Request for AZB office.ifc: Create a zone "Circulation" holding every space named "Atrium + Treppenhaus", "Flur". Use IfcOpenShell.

First a look at what the model holds.

```python
import ifcopenshell

model = ifcopenshell.open("AZB office.ifc")
print(model.schema)
seen = {}
for space in model.by_type("IfcSpace"):
    seen[space.LongName] = seen.get(space.LongName, 0) + 1
for name, count in sorted(seen.items(), key=str):
    print(count, "x", name)
print("zones:", [z.Name for z in model.by_type("IfcZone")][:20])
```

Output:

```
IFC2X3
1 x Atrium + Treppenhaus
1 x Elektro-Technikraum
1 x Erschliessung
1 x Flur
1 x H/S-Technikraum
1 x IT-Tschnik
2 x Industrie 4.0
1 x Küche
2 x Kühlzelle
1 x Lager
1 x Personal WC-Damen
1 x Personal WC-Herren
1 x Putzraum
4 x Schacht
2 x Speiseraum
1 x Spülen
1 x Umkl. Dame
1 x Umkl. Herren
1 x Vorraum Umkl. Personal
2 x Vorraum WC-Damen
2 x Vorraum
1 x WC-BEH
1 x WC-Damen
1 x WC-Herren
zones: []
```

```python
import ifcopenshell
import ifcopenshell.api.group
import ifcopenshell.api.root

model = ifcopenshell.open("AZB office.ifc")

names = {"Atrium + Treppenhaus", "Flur"}
spaces = [s for s in model.by_type("IfcSpace") if s.LongName in names]

zone = ifcopenshell.api.root.create_entity(model, ifc_class="IfcZone", name="Circulation")
ifcopenshell.api.group.assign_group(model, products=spaces, group=zone)
print(len(spaces), "spaces in", zone.Name)

model.write("AZB office_rev.ifc")
```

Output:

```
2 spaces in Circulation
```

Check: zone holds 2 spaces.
